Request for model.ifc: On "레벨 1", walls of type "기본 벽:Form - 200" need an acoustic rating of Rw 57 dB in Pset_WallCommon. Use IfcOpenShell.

First a look at what the model holds.

```python
import ifcopenshell
import ifcopenshell.util.element

model = ifcopenshell.open("model.ifc")
print(model.schema)
storey = next(s for s in model.by_type("IfcBuildingStorey") if s.Name == "레벨 1")
walls = [e for e in ifcopenshell.util.element.get_decomposition(storey) if e.is_a("IfcWall")]
seen = {}
for e in walls:
    element_type = ifcopenshell.util.element.get_type(e)
    key = (element_type.Name if element_type != e and element_type else None, ifcopenshell.util.element.get_pset(e, "Pset_WallCommon", "AcousticRating"))
    seen[key] = seen.get(key, 0) + 1
for (name, value), count in sorted(seen.items(), key=str):
    print(count, "x", name, "|", value)
```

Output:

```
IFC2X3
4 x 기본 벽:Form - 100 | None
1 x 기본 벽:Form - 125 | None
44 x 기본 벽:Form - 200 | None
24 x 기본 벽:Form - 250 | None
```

```python
import ifcopenshell
import ifcopenshell.api.pset
import ifcopenshell.util.element

model = ifcopenshell.open("model.ifc")

storey = next(s for s in model.by_type("IfcBuildingStorey") if s.Name == "레벨 1")
walls = [e for e in ifcopenshell.util.element.get_decomposition(storey) if e.is_a("IfcWall")]

count = 0
for e in walls:
    element_type = ifcopenshell.util.element.get_type(e)
    if element_type in (None, e) or element_type.Name != "기본 벽:Form - 200":
        continue
    # add_pset returns the element's existing set when there is one.
    pset = ifcopenshell.api.pset.add_pset(model, product=e, name="Pset_WallCommon")
    ifcopenshell.api.pset.edit_pset(model, pset=pset, properties={"AcousticRating": "Rw 57 dB"})
    count += 1

print(count, "walls updated")

model.write("model-out.ifc")
```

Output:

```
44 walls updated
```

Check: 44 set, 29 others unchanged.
